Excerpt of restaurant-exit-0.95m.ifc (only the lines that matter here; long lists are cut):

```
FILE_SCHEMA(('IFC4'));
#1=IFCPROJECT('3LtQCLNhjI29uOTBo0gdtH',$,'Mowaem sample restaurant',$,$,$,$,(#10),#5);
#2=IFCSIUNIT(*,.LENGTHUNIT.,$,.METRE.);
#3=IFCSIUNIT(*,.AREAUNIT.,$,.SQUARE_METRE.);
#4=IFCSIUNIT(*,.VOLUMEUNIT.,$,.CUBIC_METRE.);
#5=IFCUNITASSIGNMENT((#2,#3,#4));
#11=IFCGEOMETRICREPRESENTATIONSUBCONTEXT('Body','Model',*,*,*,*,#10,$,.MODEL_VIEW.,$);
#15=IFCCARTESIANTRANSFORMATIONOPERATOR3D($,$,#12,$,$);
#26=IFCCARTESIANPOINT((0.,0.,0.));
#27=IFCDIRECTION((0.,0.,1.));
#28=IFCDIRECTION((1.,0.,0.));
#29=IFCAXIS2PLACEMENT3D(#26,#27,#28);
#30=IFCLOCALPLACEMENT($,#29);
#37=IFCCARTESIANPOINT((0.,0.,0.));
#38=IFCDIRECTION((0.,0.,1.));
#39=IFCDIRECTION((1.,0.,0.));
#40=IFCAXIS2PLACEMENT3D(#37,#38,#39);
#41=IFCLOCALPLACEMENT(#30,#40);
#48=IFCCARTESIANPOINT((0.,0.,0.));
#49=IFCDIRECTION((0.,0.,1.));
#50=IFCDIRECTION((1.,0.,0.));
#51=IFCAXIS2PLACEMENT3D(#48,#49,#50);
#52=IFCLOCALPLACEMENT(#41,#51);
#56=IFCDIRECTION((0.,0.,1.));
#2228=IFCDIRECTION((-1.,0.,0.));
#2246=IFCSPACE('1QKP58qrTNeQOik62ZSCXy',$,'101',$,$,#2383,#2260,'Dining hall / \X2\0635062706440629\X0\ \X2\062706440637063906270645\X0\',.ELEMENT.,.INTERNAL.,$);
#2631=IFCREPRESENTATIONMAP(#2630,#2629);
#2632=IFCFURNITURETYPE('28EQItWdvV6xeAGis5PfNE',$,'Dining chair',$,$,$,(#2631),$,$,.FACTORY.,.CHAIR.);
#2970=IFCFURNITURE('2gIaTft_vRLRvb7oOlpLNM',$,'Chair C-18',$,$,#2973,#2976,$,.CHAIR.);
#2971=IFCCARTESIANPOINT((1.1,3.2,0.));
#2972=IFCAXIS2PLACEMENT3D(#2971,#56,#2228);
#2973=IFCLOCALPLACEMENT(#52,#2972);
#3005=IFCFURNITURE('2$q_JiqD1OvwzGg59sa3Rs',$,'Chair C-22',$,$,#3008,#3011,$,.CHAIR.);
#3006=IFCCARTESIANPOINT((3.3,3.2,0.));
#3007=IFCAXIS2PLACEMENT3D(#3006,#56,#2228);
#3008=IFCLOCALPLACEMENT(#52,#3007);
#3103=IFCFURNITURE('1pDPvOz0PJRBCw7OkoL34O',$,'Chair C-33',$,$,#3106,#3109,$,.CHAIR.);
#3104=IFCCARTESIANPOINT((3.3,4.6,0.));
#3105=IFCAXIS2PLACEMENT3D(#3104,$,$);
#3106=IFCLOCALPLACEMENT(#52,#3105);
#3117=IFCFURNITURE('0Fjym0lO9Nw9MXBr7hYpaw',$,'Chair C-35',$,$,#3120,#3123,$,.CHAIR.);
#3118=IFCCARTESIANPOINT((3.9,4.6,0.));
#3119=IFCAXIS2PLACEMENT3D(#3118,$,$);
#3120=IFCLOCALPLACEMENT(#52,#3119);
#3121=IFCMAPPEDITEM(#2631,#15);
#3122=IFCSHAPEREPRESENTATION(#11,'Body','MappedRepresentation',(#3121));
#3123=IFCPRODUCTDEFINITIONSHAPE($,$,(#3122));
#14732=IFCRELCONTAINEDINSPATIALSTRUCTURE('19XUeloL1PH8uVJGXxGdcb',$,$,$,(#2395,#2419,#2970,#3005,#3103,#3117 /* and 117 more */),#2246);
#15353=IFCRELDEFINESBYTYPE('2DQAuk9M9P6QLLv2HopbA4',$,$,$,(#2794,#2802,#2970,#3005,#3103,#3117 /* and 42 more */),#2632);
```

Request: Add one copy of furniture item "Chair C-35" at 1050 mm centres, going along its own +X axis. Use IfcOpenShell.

```python
import ifcopenshell
import ifcopenshell.api.geometry
import ifcopenshell.api.root
import ifcopenshell.util.element
import ifcopenshell.util.placement
import ifcopenshell.util.unit

model = ifcopenshell.open("restaurant-exit-0.95m.ifc")
unit_scale = ifcopenshell.util.unit.calculate_unit_scale(model)

source = model.by_guid("0Fjym0lO9Nw9MXBr7hYpaw")
base = ifcopenshell.util.placement.get_local_placement(source.ObjectPlacement)
step = base[:3, 0] * 1.05 / unit_scale

for i in range(1, 2):
    copy = ifcopenshell.api.root.copy_class(model, product=source)
    copy.Representation = ifcopenshell.util.element.copy_deep(
        model, source.Representation, exclude=["IfcGeometricRepresentationContext", "IfcRepresentationMap"]
    )
    matrix = base.copy()
    matrix[:3, 3] += i * step
    print("added at", matrix[:3, 3].round(3) + 0.0)
    ifcopenshell.api.geometry.edit_object_placement(model, product=copy, matrix=matrix, is_si=False)

model.write("restaurant-exit-0.95m_v2.ifc")
```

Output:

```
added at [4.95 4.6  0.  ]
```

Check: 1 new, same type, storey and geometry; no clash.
